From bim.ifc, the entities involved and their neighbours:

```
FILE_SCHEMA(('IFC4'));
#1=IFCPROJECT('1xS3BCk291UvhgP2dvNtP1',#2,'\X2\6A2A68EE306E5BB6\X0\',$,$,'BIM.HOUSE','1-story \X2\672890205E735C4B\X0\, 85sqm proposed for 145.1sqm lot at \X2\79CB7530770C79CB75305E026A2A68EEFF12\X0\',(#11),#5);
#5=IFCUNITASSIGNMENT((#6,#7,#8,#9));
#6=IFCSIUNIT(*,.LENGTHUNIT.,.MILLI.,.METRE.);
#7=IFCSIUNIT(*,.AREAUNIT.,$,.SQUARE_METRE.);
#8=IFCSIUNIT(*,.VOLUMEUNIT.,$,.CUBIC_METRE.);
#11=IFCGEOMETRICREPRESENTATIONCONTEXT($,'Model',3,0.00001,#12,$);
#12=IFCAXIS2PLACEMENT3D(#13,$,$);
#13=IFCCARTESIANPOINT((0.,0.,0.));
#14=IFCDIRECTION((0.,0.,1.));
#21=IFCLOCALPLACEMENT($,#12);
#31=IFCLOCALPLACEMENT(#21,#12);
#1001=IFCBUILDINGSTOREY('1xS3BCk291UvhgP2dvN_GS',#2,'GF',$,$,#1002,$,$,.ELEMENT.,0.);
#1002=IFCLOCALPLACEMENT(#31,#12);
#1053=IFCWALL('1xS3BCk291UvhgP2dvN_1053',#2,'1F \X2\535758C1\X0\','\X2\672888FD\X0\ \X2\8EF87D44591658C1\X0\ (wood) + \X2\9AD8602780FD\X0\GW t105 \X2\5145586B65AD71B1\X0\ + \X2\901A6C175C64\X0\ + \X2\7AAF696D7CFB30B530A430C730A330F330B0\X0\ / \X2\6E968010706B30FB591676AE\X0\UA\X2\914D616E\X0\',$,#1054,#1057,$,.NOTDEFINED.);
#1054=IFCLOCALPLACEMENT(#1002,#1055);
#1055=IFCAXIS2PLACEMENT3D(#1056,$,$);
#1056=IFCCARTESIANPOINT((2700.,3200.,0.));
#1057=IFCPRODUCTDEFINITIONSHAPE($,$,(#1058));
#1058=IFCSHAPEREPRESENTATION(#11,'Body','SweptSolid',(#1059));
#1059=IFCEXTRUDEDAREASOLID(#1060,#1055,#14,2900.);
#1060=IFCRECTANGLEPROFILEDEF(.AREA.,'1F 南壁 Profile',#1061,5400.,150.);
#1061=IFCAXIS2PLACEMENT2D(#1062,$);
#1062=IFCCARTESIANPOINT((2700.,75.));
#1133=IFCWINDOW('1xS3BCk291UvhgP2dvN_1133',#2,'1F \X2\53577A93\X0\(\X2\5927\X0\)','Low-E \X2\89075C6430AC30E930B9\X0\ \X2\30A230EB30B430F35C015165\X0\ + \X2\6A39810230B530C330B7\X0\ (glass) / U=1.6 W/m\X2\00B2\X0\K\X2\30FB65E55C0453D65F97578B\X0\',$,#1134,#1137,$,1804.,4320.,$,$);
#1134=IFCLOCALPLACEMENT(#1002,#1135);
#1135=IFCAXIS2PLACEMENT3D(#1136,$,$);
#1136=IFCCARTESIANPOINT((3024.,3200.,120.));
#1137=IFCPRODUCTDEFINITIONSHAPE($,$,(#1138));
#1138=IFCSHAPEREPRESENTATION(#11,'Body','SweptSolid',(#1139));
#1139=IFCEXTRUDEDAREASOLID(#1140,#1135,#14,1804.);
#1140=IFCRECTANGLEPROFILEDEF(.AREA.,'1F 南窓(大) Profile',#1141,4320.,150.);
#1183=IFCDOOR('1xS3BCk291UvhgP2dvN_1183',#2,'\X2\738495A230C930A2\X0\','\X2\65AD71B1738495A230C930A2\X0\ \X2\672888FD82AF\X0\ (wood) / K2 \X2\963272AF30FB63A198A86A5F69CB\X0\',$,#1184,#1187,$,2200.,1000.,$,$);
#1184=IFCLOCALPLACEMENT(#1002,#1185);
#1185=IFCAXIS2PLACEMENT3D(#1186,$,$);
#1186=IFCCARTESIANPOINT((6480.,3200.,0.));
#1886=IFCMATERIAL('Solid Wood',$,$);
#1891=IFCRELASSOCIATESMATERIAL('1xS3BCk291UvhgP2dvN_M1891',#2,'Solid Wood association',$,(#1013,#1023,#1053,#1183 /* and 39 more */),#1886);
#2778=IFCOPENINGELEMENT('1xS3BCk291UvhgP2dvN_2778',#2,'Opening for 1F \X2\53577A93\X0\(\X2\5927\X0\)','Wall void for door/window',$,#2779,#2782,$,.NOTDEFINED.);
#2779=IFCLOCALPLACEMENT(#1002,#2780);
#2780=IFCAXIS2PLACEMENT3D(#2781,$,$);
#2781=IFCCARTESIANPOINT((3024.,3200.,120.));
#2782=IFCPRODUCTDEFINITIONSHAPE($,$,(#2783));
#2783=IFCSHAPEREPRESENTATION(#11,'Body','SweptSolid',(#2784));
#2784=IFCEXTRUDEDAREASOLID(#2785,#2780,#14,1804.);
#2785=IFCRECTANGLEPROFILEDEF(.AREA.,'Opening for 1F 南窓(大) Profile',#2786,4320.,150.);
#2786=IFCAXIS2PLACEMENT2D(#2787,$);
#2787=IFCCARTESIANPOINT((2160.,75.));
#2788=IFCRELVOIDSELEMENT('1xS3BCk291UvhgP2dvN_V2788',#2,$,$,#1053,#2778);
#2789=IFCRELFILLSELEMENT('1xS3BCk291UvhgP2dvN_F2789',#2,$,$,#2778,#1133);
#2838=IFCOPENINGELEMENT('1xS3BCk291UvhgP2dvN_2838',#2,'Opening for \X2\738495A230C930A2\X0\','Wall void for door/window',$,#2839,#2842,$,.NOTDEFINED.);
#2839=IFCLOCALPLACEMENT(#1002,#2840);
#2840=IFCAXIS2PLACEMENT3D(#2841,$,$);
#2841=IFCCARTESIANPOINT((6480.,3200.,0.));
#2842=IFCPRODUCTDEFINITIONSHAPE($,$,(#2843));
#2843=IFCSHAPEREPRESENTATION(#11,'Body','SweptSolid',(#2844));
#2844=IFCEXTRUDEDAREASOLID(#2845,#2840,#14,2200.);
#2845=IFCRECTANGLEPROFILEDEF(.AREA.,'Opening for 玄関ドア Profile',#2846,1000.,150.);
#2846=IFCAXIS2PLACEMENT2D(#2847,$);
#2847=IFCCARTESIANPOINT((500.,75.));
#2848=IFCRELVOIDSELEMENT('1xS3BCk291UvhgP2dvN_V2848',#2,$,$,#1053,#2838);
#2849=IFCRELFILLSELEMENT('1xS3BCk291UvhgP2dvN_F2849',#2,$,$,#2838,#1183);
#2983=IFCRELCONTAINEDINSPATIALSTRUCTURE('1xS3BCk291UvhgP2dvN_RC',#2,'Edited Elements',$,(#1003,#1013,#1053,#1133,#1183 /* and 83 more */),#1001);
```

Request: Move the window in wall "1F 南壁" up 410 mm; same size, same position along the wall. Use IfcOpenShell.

```python
import numpy as np
import ifcopenshell
import ifcopenshell.api.geometry
import ifcopenshell.util.placement
import ifcopenshell.util.unit

model = ifcopenshell.open("bim.ifc")
unit_scale = ifcopenshell.util.unit.calculate_unit_scale(model)

window = model.by_guid("1xS3BCk291UvhgP2dvN_1133")
opening = window.FillsVoids[0].RelatingOpeningElement
dz = 410.0

shift = np.array([0.0, 0.0, dz])
# The window is not placed relative to its opening, so move both.
for product in (opening, window):
    matrix = ifcopenshell.util.placement.get_local_placement(product.ObjectPlacement)
    matrix[:3, 3] += shift
    ifcopenshell.api.geometry.edit_object_placement(model, product=product, matrix=matrix, is_si=False)

print(f"moved by {dz * unit_scale:+.3f} m")

model.write("bim_edited.ifc")
```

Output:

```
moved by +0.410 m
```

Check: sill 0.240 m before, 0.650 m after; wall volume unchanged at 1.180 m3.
